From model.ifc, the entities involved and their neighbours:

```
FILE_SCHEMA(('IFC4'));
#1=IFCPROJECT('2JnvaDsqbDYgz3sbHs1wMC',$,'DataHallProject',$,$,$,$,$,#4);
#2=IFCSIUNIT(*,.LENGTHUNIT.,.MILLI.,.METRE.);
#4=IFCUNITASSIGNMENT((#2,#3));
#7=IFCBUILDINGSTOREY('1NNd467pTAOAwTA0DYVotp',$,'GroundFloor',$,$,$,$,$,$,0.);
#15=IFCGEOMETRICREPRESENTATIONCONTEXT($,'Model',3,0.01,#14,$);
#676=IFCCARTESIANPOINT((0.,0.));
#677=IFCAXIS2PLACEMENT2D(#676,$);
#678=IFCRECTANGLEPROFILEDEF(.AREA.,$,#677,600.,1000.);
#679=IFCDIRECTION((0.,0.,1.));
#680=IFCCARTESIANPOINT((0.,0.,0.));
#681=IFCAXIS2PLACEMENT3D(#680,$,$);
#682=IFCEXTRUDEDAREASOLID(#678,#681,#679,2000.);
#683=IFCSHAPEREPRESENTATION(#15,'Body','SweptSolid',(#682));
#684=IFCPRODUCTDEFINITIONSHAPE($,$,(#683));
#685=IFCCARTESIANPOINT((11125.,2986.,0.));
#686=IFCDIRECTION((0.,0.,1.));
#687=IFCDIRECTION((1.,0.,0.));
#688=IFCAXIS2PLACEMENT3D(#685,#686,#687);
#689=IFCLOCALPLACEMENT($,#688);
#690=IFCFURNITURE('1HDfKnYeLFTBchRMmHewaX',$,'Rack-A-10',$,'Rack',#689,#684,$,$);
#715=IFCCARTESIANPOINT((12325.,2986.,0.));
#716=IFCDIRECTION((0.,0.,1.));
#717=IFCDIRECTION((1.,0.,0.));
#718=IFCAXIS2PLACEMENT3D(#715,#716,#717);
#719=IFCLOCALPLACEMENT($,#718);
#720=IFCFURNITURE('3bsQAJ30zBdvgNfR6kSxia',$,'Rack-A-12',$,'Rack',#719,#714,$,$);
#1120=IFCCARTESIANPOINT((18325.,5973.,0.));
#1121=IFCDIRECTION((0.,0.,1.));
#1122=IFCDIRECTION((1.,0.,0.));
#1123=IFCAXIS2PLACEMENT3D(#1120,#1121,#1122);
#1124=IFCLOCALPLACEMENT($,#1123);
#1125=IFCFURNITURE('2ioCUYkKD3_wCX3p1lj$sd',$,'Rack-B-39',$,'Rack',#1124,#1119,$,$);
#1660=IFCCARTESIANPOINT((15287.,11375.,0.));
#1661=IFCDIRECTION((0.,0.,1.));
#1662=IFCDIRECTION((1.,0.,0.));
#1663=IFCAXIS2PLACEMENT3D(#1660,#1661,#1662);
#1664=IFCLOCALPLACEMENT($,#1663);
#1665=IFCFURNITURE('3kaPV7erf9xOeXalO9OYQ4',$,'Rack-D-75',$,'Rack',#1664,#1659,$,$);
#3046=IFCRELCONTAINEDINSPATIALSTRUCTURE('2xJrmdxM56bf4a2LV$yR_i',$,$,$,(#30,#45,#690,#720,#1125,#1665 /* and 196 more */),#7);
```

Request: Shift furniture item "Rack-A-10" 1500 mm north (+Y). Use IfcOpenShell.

```python
import ifcopenshell
import ifcopenshell.api.geometry
import ifcopenshell.util.placement

model = ifcopenshell.open("model.ifc")

item = model.by_guid("1HDfKnYeLFTBchRMmHewaX")
matrix = ifcopenshell.util.placement.get_local_placement(item.ObjectPlacement)
matrix[1, 3] += 1500.0
ifcopenshell.api.geometry.edit_object_placement(model, product=item, matrix=matrix, is_si=False)

print(ifcopenshell.util.placement.get_local_placement(item.ObjectPlacement).round(3) + 0.0)

model.write("model_v2.ifc")
```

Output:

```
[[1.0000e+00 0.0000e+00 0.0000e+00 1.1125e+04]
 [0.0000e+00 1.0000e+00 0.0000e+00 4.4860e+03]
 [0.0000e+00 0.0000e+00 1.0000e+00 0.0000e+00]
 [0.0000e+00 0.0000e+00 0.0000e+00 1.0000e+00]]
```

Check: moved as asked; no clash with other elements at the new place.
